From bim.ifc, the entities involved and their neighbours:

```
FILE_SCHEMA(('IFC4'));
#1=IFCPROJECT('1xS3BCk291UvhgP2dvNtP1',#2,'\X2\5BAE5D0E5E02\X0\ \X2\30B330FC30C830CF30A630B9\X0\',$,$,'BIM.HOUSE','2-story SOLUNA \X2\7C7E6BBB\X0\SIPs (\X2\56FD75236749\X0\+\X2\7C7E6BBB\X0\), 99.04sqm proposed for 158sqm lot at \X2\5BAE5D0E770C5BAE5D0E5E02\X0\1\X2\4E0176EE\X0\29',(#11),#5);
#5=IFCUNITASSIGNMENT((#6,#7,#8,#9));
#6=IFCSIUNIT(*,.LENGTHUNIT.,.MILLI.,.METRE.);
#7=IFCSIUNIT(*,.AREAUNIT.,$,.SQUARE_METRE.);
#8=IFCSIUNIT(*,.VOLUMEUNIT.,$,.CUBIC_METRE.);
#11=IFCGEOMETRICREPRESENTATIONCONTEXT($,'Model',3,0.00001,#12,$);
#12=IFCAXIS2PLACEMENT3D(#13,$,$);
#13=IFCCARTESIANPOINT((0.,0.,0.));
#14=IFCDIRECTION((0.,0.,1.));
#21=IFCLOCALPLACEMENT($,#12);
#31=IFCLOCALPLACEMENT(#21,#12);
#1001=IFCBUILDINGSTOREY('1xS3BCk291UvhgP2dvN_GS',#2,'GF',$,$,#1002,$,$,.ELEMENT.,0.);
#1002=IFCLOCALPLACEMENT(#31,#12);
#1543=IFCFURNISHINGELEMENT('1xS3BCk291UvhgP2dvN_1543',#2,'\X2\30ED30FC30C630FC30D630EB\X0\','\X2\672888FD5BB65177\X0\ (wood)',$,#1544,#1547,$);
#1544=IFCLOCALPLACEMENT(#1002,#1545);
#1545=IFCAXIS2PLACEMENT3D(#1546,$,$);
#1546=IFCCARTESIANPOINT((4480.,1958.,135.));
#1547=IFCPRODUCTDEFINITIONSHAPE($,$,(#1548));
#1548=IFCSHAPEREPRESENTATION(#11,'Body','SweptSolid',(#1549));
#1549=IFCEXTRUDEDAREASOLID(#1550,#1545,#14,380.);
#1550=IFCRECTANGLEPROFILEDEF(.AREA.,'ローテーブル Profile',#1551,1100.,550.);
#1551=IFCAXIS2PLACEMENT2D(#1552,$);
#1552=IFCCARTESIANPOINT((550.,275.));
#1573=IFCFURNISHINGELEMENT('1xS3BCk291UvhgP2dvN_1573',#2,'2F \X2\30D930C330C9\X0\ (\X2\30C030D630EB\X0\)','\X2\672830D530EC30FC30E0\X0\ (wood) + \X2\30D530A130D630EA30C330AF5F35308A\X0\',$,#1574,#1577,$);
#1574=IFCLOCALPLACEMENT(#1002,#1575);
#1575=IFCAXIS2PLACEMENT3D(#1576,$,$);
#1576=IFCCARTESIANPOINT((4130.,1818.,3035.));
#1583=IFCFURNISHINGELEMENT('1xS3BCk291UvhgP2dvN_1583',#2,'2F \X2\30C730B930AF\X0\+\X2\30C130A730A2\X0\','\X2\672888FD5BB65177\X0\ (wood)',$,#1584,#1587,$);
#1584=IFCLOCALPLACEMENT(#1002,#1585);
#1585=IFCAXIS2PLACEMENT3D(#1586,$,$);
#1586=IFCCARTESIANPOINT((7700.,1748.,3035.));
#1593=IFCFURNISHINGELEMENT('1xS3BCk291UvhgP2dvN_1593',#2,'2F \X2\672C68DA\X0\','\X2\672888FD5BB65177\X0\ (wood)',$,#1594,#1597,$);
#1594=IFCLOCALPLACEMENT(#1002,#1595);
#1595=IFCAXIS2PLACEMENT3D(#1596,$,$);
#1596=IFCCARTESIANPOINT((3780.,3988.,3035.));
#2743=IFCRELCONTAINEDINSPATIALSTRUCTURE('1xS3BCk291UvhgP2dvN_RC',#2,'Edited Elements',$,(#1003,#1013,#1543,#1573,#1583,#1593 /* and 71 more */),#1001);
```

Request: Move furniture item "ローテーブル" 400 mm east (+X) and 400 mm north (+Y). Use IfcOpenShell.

```python
import ifcopenshell
import ifcopenshell.api.geometry
import ifcopenshell.util.placement

model = ifcopenshell.open("bim.ifc")

item = model.by_guid("1xS3BCk291UvhgP2dvN_1543")
matrix = ifcopenshell.util.placement.get_local_placement(item.ObjectPlacement)
matrix[0, 3] += 400.0
matrix[1, 3] += 400.0
ifcopenshell.api.geometry.edit_object_placement(model, product=item, matrix=matrix, is_si=False)

print(ifcopenshell.util.placement.get_local_placement(item.ObjectPlacement).round(3) + 0.0)

model.write("bim_updated.ifc")
```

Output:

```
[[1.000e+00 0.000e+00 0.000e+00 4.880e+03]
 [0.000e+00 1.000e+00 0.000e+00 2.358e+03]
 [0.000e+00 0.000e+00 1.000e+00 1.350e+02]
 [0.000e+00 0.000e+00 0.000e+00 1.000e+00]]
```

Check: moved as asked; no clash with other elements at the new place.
